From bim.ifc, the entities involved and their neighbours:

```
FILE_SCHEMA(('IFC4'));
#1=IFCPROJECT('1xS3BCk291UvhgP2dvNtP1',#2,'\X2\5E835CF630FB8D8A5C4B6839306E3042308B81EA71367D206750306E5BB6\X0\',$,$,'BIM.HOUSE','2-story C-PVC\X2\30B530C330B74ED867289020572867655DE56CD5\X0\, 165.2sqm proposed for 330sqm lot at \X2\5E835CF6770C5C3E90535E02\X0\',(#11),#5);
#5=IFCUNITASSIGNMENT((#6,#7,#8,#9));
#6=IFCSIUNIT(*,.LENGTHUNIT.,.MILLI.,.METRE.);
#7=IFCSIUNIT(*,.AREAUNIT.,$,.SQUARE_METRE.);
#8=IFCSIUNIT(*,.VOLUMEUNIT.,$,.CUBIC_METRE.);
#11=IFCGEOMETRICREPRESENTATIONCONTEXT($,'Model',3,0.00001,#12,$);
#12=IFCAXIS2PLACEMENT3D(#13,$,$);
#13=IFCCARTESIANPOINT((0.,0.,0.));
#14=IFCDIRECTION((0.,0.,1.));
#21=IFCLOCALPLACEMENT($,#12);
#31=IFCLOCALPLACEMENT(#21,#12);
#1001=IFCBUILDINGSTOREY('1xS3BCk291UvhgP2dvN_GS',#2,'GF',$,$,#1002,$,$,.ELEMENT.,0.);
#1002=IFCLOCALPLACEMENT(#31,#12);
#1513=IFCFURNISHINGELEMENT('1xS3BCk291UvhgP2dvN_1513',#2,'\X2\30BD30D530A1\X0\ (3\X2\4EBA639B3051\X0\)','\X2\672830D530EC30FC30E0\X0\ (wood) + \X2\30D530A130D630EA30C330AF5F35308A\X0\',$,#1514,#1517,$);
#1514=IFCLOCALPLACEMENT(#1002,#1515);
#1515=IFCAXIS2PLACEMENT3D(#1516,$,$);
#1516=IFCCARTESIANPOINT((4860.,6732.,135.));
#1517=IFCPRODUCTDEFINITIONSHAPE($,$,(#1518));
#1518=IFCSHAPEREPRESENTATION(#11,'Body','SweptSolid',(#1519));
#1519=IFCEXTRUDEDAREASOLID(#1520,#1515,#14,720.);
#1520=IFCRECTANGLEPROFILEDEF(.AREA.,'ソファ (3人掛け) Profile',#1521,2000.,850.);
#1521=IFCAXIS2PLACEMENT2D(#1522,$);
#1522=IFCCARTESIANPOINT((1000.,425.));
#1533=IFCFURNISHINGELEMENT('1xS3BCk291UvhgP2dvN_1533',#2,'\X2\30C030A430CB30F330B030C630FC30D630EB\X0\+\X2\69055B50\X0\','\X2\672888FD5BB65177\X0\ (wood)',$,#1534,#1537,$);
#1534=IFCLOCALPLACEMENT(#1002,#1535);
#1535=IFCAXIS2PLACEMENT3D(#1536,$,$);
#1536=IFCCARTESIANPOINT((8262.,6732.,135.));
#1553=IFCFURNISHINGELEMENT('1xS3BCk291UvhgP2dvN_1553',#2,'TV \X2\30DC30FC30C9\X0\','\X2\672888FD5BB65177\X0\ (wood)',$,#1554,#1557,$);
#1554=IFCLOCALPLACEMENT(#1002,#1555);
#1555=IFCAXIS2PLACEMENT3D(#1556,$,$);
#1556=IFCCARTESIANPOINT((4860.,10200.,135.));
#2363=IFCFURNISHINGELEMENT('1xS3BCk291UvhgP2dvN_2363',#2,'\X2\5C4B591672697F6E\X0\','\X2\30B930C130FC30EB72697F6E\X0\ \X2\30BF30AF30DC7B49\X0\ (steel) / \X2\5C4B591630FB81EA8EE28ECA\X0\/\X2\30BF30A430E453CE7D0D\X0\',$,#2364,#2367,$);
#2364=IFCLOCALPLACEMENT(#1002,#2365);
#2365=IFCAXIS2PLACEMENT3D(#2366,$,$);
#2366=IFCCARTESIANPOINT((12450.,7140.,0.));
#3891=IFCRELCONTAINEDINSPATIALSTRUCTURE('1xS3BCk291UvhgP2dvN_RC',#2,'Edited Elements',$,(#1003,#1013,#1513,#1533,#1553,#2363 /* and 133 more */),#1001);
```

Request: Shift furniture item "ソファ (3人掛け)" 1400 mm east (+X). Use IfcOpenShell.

```python
import ifcopenshell
import ifcopenshell.api.geometry
import ifcopenshell.util.placement
import ifcopenshell.util.unit

model = ifcopenshell.open("bim.ifc")
unit_scale = ifcopenshell.util.unit.calculate_unit_scale(model)

item = model.by_guid("1xS3BCk291UvhgP2dvN_1513")
matrix = ifcopenshell.util.placement.get_local_placement(item.ObjectPlacement)
matrix[0, 3] += 1.4 / unit_scale
ifcopenshell.api.geometry.edit_object_placement(model, product=item, matrix=matrix, is_si=False)

print(ifcopenshell.util.placement.get_local_placement(item.ObjectPlacement).round(3) + 0.0)

model.write("bim_v2.ifc")
```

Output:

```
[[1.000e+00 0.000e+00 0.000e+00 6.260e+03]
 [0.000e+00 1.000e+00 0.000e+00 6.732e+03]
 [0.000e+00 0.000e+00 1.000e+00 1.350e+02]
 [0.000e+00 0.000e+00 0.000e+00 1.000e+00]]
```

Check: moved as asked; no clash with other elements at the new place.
